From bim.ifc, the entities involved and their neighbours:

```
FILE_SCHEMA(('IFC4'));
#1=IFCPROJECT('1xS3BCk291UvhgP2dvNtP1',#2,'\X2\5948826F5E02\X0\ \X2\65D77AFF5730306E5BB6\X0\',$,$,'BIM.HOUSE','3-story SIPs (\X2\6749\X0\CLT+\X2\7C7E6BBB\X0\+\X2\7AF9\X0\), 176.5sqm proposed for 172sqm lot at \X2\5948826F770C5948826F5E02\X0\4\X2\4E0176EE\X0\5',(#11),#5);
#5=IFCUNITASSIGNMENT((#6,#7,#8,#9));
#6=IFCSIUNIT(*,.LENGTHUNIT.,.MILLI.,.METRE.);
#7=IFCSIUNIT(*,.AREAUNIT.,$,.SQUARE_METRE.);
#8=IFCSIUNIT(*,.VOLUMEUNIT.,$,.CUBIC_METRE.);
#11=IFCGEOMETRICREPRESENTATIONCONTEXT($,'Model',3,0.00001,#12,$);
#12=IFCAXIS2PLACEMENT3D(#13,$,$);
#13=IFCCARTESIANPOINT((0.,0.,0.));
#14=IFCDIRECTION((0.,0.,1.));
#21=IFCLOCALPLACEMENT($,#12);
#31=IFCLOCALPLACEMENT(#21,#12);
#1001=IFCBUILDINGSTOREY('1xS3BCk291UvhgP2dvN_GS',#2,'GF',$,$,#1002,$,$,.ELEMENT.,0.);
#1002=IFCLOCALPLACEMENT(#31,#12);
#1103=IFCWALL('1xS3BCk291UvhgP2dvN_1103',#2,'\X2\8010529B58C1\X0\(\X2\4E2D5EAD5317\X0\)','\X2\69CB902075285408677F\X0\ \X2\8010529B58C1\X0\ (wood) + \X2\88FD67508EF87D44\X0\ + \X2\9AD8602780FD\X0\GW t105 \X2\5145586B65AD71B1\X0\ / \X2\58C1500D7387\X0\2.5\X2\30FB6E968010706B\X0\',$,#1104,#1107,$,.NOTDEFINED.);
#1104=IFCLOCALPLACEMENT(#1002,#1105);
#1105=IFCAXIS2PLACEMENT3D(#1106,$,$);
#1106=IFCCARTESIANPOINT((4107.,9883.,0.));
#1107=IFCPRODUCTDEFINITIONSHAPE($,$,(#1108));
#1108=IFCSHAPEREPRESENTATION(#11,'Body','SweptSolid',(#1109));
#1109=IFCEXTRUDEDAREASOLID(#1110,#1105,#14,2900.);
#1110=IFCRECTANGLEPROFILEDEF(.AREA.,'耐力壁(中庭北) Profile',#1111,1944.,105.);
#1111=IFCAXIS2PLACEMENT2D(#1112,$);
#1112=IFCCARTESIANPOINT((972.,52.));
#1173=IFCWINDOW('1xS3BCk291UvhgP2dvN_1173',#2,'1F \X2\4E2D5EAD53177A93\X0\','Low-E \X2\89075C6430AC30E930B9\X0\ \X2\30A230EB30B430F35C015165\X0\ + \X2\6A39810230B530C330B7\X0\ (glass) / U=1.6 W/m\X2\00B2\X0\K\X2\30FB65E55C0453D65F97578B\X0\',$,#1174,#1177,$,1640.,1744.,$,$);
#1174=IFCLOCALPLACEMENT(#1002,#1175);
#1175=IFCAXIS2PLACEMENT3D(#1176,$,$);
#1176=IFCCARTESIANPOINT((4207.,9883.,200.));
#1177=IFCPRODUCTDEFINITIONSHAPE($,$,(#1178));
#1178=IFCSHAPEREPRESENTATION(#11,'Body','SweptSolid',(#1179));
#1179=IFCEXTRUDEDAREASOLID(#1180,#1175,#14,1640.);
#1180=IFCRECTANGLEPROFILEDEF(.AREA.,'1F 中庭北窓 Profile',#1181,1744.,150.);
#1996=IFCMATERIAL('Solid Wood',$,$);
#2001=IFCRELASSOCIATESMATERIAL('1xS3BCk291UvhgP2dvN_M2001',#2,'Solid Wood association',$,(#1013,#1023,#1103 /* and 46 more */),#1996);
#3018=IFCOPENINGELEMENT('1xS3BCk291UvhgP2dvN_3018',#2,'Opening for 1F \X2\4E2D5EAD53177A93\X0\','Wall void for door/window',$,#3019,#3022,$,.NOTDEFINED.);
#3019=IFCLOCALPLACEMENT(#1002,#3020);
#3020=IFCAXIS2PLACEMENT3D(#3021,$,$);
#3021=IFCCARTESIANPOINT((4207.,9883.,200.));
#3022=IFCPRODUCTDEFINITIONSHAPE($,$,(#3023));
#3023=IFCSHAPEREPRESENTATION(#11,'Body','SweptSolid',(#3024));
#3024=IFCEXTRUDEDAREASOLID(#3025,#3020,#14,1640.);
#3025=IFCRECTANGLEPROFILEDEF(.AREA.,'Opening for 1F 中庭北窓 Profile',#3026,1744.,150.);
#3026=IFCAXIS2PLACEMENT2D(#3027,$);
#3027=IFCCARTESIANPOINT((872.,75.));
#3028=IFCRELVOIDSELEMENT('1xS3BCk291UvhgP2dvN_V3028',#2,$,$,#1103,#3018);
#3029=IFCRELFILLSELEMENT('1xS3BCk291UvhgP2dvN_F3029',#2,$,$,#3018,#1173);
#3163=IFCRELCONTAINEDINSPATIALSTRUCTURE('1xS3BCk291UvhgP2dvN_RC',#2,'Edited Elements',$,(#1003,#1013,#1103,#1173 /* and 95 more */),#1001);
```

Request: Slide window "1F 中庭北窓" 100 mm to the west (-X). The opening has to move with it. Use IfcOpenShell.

```python
import ifcopenshell
import ifcopenshell.api.geometry
import ifcopenshell.util.placement

model = ifcopenshell.open("bim.ifc")

window = model.by_guid("1xS3BCk291UvhgP2dvN_1173")
opening = window.FillsVoids[0].RelatingOpeningElement
wall = opening.VoidsElements[0].RelatingBuildingElement

wall_matrix = ifcopenshell.util.placement.get_local_placement(wall.ObjectPlacement)
shift = wall_matrix[:3, 0] * -100.0
before = ifcopenshell.util.placement.get_local_placement(window.ObjectPlacement)[:3, 3].copy()

# The window is not placed relative to its opening, so move both.
for product in (opening, window):
    matrix = ifcopenshell.util.placement.get_local_placement(product.ObjectPlacement)
    matrix[:3, 3] += shift
    ifcopenshell.api.geometry.edit_object_placement(model, product=product, matrix=matrix, is_si=False)

after = ifcopenshell.util.placement.get_local_placement(window.ObjectPlacement)[:3, 3]
print("window moved by", (after - before).round(3) + 0.0)

model.write("bim_rev.ifc")
```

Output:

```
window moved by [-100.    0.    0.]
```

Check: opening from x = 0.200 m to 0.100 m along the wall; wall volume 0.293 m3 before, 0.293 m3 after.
